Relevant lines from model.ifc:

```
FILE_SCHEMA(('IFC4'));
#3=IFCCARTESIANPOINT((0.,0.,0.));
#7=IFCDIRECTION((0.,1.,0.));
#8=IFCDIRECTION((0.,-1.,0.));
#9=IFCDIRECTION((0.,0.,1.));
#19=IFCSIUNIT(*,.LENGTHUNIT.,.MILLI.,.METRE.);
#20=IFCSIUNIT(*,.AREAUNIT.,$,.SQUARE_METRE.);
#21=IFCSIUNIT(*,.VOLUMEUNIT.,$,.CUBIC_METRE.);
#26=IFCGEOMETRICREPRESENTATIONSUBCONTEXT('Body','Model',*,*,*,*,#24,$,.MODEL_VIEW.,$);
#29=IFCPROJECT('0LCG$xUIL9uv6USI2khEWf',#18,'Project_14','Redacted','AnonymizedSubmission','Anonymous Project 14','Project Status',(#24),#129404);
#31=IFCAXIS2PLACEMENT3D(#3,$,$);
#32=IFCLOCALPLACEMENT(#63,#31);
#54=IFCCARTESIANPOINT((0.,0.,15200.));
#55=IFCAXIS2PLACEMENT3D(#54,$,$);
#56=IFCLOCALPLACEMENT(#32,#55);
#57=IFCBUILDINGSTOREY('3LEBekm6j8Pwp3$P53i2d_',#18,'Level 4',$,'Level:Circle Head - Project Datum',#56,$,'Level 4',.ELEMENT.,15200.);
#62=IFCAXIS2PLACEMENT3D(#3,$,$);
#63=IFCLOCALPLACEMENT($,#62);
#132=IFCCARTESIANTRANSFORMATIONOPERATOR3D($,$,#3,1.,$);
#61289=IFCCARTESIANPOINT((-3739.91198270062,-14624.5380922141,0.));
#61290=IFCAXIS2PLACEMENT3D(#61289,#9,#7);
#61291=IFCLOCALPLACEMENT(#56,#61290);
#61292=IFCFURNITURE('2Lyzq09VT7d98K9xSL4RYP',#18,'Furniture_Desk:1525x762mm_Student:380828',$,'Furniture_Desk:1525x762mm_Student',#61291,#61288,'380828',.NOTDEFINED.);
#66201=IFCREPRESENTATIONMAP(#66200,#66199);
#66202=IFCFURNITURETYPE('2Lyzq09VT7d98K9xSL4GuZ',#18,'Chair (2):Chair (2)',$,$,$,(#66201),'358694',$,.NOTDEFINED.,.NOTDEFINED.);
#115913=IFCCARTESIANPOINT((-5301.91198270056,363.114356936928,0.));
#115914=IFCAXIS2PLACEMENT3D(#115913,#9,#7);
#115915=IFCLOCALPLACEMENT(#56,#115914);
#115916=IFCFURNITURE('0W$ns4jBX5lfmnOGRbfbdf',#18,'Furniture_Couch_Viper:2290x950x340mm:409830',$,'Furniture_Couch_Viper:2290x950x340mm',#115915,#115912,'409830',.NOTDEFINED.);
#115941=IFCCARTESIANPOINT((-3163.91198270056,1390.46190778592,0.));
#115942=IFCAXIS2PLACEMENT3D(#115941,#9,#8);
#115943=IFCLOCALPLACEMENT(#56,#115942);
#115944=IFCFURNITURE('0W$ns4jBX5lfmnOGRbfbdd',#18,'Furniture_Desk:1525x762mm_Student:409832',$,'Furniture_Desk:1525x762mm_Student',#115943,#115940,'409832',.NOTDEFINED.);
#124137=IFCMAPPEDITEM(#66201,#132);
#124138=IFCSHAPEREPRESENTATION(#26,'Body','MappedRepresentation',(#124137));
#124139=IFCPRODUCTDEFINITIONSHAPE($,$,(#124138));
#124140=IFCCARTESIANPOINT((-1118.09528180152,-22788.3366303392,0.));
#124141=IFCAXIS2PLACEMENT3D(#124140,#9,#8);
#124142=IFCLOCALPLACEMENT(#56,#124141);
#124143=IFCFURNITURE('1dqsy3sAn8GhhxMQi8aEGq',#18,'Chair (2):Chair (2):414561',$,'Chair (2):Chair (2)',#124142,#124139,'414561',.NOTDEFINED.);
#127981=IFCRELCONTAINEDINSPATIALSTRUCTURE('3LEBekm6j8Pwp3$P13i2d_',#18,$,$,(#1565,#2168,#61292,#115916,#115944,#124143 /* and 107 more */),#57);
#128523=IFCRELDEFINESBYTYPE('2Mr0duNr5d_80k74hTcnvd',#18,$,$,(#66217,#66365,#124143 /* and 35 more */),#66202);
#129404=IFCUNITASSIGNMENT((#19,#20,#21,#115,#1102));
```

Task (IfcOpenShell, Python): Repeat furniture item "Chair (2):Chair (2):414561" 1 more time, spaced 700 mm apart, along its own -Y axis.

```python
import ifcopenshell
import ifcopenshell.api.geometry
import ifcopenshell.api.root
import ifcopenshell.util.element
import ifcopenshell.util.placement
import ifcopenshell.util.unit

model = ifcopenshell.open("model.ifc")
unit_scale = ifcopenshell.util.unit.calculate_unit_scale(model)


def reuse_history(source, copy):
    """copy_class also copies each property set's owner history, people and application; keep the originals."""
    for rel in copy.IsDefinedBy:
        if rel.is_a("IfcRelDefinesByProperties") and (history := rel.RelatingPropertyDefinition.OwnerHistory):
            rel.RelatingPropertyDefinition.OwnerHistory = source.OwnerHistory
            ifcopenshell.util.element.remove_deep2(model, history)


source = model.by_guid("1dqsy3sAn8GhhxMQi8aEGq")
base = ifcopenshell.util.placement.get_local_placement(source.ObjectPlacement)
step = -base[:3, 1] * 0.7 / unit_scale

for i in range(1, 2):
    copy = ifcopenshell.api.root.copy_class(model, product=source)
    copy.Representation = ifcopenshell.util.element.copy_deep(
        model, source.Representation, exclude=["IfcGeometricRepresentationContext", "IfcRepresentationMap"]
    )
    copy.Name = "Chair (2):Chair (2)"
    copy.Tag = None
    reuse_history(source, copy)
    matrix = base.copy()
    matrix[:3, 3] += i * step
    print("added at", matrix[:3, 3].round(3) + 0.0)
    ifcopenshell.api.geometry.edit_object_placement(model, product=copy, matrix=matrix, is_si=False)

model.write("model-out.ifc")
```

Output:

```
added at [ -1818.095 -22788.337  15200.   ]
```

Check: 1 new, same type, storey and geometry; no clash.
